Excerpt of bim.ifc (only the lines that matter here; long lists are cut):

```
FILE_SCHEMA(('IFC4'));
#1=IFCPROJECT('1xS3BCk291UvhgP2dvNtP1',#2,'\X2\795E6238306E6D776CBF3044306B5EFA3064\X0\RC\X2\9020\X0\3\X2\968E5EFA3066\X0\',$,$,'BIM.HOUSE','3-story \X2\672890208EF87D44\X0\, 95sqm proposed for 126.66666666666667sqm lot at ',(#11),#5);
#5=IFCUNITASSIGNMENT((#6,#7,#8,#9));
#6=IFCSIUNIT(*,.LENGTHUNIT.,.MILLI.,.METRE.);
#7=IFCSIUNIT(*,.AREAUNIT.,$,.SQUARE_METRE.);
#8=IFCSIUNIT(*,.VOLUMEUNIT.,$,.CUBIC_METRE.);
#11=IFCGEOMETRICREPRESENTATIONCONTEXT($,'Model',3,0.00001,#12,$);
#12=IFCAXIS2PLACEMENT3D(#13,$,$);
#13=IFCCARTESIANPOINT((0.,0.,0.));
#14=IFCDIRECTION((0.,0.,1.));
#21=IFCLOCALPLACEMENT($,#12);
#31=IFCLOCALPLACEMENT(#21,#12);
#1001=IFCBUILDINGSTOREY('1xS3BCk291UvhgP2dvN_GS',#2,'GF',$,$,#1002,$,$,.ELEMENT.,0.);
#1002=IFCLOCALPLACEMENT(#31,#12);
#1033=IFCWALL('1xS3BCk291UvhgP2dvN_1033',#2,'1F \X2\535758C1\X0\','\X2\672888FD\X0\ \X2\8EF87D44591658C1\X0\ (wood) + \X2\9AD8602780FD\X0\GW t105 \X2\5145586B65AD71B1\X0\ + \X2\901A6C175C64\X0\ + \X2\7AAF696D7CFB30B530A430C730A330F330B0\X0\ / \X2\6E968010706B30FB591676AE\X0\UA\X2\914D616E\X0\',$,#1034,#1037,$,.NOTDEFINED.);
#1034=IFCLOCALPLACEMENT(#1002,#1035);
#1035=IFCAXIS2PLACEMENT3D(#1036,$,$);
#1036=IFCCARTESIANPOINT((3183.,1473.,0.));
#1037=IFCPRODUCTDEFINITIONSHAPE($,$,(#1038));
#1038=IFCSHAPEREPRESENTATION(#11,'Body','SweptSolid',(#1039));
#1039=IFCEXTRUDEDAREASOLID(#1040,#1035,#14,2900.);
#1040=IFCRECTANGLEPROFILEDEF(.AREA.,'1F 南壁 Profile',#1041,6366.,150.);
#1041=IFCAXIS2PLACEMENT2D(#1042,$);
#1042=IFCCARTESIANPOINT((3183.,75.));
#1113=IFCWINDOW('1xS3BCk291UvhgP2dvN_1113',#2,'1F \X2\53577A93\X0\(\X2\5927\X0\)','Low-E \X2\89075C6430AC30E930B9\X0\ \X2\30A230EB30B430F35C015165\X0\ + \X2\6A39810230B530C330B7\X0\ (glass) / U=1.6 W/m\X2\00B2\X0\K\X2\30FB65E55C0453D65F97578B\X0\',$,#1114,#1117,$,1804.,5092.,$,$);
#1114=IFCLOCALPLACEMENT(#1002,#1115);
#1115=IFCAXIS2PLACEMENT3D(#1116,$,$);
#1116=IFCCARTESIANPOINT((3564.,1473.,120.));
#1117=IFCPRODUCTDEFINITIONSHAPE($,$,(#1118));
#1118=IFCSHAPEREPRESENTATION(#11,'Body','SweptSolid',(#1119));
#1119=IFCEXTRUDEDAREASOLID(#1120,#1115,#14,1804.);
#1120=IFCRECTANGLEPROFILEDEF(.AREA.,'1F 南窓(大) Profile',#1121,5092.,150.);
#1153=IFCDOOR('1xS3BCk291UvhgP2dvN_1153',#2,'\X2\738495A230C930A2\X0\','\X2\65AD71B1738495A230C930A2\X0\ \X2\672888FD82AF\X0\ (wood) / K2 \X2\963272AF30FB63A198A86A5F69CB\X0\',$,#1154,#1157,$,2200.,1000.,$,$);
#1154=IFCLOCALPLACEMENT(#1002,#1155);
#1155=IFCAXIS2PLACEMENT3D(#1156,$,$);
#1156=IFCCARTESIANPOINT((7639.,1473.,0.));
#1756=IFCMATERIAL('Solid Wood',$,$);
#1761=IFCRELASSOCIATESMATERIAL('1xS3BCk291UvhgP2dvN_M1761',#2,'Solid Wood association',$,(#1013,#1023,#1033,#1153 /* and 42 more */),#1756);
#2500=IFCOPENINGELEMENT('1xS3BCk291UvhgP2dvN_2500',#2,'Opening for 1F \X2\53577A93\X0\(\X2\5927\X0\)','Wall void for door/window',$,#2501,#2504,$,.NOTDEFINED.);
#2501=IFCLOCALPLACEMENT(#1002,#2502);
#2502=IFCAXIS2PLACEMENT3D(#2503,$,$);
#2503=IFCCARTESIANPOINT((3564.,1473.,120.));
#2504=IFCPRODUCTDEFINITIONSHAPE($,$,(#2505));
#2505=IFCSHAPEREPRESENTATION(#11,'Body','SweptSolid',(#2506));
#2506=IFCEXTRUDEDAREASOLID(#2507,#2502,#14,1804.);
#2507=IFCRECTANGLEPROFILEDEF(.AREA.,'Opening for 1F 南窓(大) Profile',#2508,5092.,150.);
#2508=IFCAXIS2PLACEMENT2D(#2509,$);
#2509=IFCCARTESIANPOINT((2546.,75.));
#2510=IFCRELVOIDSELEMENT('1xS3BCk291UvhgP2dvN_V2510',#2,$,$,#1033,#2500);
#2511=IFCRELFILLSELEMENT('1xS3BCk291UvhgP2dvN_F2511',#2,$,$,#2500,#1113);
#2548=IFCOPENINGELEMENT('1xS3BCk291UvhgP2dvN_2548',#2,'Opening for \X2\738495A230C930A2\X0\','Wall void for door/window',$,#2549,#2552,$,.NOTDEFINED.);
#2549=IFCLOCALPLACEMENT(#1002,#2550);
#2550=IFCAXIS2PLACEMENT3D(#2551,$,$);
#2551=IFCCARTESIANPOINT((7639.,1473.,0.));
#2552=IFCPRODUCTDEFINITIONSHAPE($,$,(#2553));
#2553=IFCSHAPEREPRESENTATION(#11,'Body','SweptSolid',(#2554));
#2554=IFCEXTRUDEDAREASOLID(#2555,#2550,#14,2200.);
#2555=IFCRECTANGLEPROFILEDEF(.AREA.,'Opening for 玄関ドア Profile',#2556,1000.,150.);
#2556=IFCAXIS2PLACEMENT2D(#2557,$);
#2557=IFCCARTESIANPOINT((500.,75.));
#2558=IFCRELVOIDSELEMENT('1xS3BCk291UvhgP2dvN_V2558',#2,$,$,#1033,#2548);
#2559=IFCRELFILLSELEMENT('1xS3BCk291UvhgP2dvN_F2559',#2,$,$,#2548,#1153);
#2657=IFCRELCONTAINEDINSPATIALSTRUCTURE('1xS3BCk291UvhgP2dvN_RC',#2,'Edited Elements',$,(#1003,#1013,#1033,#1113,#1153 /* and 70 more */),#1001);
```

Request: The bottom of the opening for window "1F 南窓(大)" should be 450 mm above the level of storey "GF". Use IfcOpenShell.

```python
import numpy as np
import ifcopenshell
import ifcopenshell.api.geometry
import ifcopenshell.geom
import ifcopenshell.util.element
import ifcopenshell.util.placement
import ifcopenshell.util.shape
import ifcopenshell.util.unit

model = ifcopenshell.open("bim.ifc")
unit_scale = ifcopenshell.util.unit.calculate_unit_scale(model)

window = model.by_guid("1xS3BCk291UvhgP2dvN_1113")
opening = window.FillsVoids[0].RelatingOpeningElement
storey = ifcopenshell.util.element.get_container(window, ifc_class="IfcBuildingStorey")
level = ifcopenshell.util.placement.get_local_placement(storey.ObjectPlacement)[2, 3]

# The opening's origin need not be at the sill, so measure its lowest point.
shape = ifcopenshell.geom.create_shape(ifcopenshell.geom.settings(), opening)
bottom = ifcopenshell.util.shape.get_shape_bottom_elevation(shape, shape.geometry) / unit_scale
dz = level + 450.0 - bottom

shift = np.array([0.0, 0.0, dz])
# The window is not placed relative to its opening, so move both.
for product in (opening, window):
    matrix = ifcopenshell.util.placement.get_local_placement(product.ObjectPlacement)
    matrix[:3, 3] += shift
    ifcopenshell.api.geometry.edit_object_placement(model, product=product, matrix=matrix, is_si=False)

print(f"moved by {dz * unit_scale:+.3f} m")

model.write("bim-out.ifc")
```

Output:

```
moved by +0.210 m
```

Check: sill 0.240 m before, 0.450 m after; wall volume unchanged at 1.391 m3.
